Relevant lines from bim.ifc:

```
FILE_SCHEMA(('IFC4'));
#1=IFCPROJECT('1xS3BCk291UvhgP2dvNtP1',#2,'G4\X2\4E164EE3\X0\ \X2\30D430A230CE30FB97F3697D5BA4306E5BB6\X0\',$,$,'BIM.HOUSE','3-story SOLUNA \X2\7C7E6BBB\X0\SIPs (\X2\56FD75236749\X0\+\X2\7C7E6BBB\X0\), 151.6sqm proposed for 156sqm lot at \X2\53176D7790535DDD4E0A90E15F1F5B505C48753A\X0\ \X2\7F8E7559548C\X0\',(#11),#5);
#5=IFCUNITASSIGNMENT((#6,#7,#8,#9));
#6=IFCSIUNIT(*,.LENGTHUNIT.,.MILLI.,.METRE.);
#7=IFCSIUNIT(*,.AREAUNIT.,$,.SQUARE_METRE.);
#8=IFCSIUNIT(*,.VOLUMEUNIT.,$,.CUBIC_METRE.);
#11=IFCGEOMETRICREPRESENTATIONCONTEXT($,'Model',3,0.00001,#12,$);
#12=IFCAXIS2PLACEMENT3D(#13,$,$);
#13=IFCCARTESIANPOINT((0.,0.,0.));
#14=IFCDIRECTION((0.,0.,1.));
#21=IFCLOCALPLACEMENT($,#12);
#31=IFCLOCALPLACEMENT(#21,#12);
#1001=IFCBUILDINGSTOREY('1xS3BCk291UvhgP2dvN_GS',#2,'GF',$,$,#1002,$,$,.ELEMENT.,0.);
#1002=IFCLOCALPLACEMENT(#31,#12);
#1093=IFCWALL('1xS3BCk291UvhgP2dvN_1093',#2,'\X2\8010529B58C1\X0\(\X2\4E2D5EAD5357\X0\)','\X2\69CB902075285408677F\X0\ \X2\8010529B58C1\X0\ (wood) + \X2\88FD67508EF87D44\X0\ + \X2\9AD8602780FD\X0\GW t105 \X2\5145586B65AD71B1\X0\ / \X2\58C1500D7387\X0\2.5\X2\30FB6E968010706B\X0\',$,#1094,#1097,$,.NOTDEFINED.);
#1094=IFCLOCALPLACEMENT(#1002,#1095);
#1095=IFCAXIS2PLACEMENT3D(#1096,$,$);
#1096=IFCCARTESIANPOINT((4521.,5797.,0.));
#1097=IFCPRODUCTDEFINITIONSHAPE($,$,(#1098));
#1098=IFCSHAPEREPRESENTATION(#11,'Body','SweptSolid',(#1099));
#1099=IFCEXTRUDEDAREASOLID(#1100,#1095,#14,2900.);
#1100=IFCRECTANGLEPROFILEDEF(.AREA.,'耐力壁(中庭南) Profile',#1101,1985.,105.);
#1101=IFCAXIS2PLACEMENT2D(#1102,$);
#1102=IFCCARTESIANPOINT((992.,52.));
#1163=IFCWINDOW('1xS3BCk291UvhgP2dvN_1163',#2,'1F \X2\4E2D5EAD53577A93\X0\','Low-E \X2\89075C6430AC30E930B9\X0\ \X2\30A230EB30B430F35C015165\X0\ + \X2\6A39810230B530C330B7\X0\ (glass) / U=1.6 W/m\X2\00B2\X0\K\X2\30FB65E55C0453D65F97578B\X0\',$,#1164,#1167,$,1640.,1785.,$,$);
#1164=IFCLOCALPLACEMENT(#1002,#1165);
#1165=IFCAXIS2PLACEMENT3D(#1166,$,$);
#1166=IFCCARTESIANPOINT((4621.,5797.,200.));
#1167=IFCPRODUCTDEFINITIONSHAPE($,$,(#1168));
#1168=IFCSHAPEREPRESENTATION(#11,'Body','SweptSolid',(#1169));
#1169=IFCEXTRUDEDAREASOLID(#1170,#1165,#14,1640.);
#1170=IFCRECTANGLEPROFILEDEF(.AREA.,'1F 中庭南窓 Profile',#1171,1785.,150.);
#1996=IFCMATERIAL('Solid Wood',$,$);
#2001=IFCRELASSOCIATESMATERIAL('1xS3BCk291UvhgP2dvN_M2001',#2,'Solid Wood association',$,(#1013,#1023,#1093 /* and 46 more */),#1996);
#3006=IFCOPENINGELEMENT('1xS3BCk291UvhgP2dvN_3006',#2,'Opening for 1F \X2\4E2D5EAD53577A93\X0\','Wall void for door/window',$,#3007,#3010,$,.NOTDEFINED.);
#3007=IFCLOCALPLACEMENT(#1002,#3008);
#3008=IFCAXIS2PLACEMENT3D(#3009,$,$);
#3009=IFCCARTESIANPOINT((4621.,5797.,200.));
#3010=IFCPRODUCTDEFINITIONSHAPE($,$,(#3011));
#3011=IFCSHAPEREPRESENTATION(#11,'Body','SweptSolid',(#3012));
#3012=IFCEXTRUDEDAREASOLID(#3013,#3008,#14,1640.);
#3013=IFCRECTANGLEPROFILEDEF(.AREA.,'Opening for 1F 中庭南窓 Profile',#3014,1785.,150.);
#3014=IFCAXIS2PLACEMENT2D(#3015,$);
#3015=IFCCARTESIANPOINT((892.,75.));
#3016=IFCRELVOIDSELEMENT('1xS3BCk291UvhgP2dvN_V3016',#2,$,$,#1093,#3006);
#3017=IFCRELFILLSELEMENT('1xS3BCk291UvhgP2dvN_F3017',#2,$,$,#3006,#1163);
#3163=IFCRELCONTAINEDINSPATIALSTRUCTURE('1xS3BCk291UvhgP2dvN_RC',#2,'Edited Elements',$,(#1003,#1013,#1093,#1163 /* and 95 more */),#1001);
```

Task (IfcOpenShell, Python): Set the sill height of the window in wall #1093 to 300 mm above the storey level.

```python
import numpy as np
import ifcopenshell
import ifcopenshell.api.geometry
import ifcopenshell.geom
import ifcopenshell.util.element
import ifcopenshell.util.placement
import ifcopenshell.util.shape
import ifcopenshell.util.unit

model = ifcopenshell.open("bim.ifc")
unit_scale = ifcopenshell.util.unit.calculate_unit_scale(model)

window = model.by_id(1163)
opening = window.FillsVoids[0].RelatingOpeningElement
storey = ifcopenshell.util.element.get_container(window, ifc_class="IfcBuildingStorey")
level = ifcopenshell.util.placement.get_local_placement(storey.ObjectPlacement)[2, 3]

# The opening's origin need not be at the sill, so measure its lowest point.
shape = ifcopenshell.geom.create_shape(ifcopenshell.geom.settings(), opening)
bottom = ifcopenshell.util.shape.get_shape_bottom_elevation(shape, shape.geometry) / unit_scale
dz = level + 0.3 / unit_scale - bottom

shift = np.array([0.0, 0.0, dz])
# The window is not placed relative to its opening, so move both.
for product in (opening, window):
    matrix = ifcopenshell.util.placement.get_local_placement(product.ObjectPlacement)
    matrix[:3, 3] += shift
    ifcopenshell.api.geometry.edit_object_placement(model, product=product, matrix=matrix, is_si=False)

print(f"moved by {dz * unit_scale:+.3f} m")

model.write("bim_rev.ifc")
```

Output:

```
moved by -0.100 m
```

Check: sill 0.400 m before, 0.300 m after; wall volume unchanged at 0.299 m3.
